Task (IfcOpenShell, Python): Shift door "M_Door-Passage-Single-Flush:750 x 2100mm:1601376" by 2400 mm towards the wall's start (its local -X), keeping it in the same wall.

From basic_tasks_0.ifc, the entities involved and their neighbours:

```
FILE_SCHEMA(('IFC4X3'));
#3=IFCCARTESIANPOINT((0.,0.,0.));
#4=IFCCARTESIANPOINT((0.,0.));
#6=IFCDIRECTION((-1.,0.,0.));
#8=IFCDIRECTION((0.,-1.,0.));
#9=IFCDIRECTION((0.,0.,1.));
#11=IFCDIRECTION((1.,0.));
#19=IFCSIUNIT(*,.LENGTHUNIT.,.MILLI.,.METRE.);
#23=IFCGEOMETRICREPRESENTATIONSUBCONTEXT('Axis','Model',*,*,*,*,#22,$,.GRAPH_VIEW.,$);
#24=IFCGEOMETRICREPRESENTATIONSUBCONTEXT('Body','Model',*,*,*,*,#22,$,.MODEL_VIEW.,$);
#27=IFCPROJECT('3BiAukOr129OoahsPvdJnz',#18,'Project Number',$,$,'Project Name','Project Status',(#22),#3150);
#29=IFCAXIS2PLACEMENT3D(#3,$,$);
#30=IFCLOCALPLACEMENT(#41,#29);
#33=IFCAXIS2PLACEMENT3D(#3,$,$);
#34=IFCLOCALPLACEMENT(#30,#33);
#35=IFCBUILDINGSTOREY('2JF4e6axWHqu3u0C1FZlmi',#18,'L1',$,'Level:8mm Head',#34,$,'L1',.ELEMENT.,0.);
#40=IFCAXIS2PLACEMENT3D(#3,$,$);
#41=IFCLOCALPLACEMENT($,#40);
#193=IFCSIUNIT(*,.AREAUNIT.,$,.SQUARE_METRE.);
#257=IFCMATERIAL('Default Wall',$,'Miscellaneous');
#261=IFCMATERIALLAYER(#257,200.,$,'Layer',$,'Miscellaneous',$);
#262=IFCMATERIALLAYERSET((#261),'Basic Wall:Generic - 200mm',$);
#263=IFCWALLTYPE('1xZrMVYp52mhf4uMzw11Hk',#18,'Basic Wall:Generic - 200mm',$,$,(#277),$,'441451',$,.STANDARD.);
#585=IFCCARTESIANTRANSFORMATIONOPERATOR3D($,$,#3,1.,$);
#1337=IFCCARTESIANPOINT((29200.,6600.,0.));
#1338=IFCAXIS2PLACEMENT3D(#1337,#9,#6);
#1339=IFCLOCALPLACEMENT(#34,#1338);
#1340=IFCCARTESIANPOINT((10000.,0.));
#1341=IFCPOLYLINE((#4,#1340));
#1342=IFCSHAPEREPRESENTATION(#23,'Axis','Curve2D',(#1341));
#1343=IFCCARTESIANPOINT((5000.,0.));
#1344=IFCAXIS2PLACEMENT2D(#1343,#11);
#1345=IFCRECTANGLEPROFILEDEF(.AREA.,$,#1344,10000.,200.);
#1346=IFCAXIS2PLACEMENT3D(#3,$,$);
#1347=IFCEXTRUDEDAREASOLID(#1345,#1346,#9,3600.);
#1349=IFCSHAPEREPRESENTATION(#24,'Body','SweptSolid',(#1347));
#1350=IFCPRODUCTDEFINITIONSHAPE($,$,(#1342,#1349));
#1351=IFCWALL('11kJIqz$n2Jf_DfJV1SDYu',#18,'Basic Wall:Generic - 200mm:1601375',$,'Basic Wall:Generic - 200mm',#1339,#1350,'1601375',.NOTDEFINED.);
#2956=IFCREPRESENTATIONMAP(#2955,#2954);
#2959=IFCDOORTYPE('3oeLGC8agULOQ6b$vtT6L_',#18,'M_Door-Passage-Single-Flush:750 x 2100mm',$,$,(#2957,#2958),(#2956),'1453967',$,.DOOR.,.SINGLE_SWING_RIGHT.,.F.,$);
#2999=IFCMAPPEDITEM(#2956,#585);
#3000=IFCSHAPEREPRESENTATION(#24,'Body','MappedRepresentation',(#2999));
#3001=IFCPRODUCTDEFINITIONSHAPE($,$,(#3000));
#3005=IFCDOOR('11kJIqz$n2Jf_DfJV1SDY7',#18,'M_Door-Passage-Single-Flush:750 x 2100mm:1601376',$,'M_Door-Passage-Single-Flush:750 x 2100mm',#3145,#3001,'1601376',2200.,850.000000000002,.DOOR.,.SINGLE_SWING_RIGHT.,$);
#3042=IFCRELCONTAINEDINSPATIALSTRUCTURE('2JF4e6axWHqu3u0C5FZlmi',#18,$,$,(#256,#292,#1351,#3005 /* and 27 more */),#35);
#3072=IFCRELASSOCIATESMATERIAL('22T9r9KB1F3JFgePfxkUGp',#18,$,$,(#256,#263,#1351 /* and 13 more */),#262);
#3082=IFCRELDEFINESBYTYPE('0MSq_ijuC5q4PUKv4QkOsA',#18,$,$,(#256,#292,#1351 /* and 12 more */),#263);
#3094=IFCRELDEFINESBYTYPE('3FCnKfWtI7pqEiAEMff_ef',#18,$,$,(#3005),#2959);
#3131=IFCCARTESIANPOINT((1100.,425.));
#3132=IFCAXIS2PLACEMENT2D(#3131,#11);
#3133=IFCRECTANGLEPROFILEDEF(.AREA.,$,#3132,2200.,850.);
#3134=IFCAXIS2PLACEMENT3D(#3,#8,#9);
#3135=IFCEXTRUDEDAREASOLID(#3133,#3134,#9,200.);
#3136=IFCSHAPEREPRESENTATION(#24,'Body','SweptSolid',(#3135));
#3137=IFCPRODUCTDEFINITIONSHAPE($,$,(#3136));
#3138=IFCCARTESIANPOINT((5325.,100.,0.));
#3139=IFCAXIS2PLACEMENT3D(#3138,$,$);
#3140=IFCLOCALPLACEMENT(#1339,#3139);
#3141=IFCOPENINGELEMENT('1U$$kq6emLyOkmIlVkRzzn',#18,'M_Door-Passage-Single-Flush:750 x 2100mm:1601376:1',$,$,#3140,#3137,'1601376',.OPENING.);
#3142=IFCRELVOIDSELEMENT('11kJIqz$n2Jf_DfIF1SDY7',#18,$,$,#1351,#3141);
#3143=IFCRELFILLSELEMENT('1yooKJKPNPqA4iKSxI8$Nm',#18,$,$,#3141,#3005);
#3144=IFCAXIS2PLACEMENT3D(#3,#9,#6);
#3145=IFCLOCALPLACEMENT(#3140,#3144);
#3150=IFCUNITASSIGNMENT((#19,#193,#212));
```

```python
import ifcopenshell
import ifcopenshell.api.geometry
import ifcopenshell.util.placement
import ifcopenshell.util.unit

model = ifcopenshell.open("basic_tasks_0.ifc")
unit_scale = ifcopenshell.util.unit.calculate_unit_scale(model)

door = model.by_guid("11kJIqz$n2Jf_DfJV1SDY7")
opening = door.FillsVoids[0].RelatingOpeningElement
wall = opening.VoidsElements[0].RelatingBuildingElement

wall_matrix = ifcopenshell.util.placement.get_local_placement(wall.ObjectPlacement)
shift = wall_matrix[:3, 0] * -2.4 / unit_scale
before = ifcopenshell.util.placement.get_local_placement(door.ObjectPlacement)[:3, 3].copy()

# The door is placed relative to its opening, so it follows when the opening moves.
matrix = ifcopenshell.util.placement.get_local_placement(opening.ObjectPlacement)
matrix[:3, 3] += shift
ifcopenshell.api.geometry.edit_object_placement(
    model, product=opening, matrix=matrix, is_si=False, should_transform_children=True
)

after = ifcopenshell.util.placement.get_local_placement(door.ObjectPlacement)[:3, 3]
print("door moved by", (after - before).round(3) + 0.0)

model.write("basic_tasks_0_v2.ifc")
```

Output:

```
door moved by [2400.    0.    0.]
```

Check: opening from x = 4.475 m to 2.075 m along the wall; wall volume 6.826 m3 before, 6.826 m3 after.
